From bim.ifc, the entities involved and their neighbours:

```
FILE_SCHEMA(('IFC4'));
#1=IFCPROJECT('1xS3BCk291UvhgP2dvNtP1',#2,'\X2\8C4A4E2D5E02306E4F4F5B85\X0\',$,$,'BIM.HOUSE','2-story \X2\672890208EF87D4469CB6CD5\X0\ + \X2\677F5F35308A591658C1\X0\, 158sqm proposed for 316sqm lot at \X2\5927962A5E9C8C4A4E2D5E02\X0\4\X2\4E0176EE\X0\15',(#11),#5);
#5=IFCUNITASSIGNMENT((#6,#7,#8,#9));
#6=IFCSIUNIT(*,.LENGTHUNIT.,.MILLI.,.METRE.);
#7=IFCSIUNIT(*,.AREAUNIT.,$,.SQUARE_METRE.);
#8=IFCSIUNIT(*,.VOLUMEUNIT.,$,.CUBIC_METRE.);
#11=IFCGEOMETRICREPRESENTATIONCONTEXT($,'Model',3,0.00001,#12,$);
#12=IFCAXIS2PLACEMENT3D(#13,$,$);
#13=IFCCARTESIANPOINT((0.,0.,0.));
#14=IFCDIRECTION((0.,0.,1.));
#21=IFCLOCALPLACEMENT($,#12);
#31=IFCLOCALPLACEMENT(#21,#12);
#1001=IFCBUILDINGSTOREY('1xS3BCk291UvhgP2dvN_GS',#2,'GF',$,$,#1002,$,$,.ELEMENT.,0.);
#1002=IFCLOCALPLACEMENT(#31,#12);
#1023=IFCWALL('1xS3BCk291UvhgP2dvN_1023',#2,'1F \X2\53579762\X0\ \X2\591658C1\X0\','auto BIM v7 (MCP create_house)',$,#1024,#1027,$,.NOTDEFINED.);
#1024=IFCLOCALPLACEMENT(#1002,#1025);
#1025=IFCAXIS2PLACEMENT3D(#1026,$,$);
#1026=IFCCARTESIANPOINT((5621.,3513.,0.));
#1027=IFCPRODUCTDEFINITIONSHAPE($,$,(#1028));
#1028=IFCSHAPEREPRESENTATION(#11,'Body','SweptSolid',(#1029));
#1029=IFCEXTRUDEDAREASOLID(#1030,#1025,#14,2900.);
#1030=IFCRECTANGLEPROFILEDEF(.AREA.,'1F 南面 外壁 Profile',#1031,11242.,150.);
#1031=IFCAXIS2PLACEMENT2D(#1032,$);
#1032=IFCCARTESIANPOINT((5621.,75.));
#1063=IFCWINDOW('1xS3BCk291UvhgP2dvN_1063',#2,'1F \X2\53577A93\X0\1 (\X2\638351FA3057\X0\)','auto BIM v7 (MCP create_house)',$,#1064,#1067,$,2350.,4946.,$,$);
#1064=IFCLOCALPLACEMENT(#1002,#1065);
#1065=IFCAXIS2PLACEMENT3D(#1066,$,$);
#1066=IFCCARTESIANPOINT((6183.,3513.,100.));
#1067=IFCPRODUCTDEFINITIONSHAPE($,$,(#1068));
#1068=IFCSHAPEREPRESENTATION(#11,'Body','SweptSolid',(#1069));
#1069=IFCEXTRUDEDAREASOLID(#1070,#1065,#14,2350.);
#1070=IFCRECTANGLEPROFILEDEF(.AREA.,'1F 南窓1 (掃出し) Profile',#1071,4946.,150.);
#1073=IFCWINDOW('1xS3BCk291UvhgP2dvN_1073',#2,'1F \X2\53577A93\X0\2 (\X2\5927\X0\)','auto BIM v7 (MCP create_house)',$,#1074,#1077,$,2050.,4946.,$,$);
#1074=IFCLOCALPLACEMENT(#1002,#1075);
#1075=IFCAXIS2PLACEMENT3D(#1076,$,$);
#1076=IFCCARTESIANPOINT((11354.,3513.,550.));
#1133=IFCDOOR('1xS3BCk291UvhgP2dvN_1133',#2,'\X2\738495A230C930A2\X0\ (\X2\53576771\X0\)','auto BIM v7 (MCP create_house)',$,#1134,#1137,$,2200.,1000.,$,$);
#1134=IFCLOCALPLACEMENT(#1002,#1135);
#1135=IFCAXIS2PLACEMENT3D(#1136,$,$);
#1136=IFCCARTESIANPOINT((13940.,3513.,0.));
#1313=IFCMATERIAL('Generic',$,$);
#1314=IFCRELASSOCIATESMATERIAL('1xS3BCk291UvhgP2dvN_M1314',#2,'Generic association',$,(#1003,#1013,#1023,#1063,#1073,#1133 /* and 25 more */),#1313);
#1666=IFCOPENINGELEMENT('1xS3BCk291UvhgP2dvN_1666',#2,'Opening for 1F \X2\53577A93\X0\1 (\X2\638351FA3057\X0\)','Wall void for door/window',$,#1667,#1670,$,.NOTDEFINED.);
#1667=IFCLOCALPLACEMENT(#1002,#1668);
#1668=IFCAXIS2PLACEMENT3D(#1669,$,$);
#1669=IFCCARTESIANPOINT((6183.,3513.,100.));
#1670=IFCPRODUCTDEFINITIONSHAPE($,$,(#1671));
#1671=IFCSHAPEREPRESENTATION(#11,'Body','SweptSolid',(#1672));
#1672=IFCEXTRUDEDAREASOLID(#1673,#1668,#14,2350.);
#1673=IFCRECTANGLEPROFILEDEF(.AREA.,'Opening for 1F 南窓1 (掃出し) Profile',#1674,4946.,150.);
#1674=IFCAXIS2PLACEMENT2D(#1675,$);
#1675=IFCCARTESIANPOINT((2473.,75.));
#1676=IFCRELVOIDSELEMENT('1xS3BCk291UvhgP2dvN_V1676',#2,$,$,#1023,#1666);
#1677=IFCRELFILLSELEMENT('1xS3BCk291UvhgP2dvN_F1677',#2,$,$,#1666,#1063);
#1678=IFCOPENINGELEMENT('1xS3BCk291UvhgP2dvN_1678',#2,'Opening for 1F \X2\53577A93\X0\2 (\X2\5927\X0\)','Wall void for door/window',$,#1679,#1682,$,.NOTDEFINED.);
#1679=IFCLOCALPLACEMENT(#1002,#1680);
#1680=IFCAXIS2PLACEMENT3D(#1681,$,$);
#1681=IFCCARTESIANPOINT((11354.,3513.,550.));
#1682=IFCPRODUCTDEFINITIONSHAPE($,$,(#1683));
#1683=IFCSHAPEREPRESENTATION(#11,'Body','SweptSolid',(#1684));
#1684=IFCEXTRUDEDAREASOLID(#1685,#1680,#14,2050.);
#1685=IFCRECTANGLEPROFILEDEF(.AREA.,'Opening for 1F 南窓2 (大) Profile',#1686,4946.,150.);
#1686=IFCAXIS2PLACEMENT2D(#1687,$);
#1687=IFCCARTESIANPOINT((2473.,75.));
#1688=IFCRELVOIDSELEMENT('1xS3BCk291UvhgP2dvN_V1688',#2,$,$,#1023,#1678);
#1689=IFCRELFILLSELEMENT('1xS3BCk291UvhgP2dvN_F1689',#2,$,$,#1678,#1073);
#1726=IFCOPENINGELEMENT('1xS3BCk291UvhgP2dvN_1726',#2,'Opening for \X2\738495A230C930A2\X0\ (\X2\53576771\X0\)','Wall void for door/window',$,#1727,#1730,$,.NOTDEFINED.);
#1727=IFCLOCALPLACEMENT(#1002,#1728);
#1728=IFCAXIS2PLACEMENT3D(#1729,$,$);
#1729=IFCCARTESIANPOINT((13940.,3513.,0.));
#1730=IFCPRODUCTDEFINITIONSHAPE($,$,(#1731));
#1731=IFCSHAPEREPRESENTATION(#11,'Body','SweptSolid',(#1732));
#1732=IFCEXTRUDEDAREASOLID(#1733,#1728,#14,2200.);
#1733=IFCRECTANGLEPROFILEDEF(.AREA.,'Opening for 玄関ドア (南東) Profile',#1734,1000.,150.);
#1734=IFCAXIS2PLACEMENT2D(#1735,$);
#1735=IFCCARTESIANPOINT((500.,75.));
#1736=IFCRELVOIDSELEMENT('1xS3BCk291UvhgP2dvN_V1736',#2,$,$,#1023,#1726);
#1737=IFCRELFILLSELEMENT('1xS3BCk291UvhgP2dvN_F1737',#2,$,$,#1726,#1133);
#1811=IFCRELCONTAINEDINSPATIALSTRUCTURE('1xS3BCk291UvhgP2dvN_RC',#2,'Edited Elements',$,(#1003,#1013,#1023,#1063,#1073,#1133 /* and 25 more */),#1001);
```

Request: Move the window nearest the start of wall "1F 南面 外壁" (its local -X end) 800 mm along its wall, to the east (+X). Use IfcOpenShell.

```python
import ifcopenshell
import ifcopenshell.api.geometry
import ifcopenshell.util.placement
import ifcopenshell.util.unit

model = ifcopenshell.open("bim.ifc")
unit_scale = ifcopenshell.util.unit.calculate_unit_scale(model)

window = model.by_guid("1xS3BCk291UvhgP2dvN_1063")
opening = window.FillsVoids[0].RelatingOpeningElement
wall = opening.VoidsElements[0].RelatingBuildingElement

wall_matrix = ifcopenshell.util.placement.get_local_placement(wall.ObjectPlacement)
shift = wall_matrix[:3, 0] * 0.8 / unit_scale
before = ifcopenshell.util.placement.get_local_placement(window.ObjectPlacement)[:3, 3].copy()

# The window is not placed relative to its opening, so move both.
for product in (opening, window):
    matrix = ifcopenshell.util.placement.get_local_placement(product.ObjectPlacement)
    matrix[:3, 3] += shift
    ifcopenshell.api.geometry.edit_object_placement(model, product=product, matrix=matrix, is_si=False)

after = ifcopenshell.util.placement.get_local_placement(window.ObjectPlacement)[:3, 3]
print("window moved by", (after - before).round(3) + 0.0)

model.write("bim-out.ifc")
```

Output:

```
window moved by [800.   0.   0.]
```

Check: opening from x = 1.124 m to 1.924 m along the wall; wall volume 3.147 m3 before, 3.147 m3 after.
